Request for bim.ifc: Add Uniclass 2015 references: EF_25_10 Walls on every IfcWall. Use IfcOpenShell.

First a look at what the model holds.

```python
import ifcopenshell

model = ifcopenshell.open("bim.ifc")
print(model.schema)
print("classifications:", [c.Name for c in model.by_type("IfcClassification")])
for ifc_class in ("IfcDoor", "IfcRoof", "IfcStair", "IfcWall", "IfcWindow"):
    print(ifc_class, len(model.by_type(ifc_class)))
```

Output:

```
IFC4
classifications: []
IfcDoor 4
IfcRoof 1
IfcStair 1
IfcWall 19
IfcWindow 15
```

```python
import ifcopenshell
import ifcopenshell.api.classification

model = ifcopenshell.open("bim.ifc")

system = ifcopenshell.api.classification.add_classification(model, classification="Uniclass 2015")

codes = {
    "IfcWall": ("EF_25_10", "Walls"),
}
for ifc_class, (code, name) in codes.items():
    products = model.by_type(ifc_class)
    ifcopenshell.api.classification.add_reference(
        model, products=products, classification=system, identification=code, name=name
    )
    print(code, len(products))

model.write("bim_rev.ifc")
```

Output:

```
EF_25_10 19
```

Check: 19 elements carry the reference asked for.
